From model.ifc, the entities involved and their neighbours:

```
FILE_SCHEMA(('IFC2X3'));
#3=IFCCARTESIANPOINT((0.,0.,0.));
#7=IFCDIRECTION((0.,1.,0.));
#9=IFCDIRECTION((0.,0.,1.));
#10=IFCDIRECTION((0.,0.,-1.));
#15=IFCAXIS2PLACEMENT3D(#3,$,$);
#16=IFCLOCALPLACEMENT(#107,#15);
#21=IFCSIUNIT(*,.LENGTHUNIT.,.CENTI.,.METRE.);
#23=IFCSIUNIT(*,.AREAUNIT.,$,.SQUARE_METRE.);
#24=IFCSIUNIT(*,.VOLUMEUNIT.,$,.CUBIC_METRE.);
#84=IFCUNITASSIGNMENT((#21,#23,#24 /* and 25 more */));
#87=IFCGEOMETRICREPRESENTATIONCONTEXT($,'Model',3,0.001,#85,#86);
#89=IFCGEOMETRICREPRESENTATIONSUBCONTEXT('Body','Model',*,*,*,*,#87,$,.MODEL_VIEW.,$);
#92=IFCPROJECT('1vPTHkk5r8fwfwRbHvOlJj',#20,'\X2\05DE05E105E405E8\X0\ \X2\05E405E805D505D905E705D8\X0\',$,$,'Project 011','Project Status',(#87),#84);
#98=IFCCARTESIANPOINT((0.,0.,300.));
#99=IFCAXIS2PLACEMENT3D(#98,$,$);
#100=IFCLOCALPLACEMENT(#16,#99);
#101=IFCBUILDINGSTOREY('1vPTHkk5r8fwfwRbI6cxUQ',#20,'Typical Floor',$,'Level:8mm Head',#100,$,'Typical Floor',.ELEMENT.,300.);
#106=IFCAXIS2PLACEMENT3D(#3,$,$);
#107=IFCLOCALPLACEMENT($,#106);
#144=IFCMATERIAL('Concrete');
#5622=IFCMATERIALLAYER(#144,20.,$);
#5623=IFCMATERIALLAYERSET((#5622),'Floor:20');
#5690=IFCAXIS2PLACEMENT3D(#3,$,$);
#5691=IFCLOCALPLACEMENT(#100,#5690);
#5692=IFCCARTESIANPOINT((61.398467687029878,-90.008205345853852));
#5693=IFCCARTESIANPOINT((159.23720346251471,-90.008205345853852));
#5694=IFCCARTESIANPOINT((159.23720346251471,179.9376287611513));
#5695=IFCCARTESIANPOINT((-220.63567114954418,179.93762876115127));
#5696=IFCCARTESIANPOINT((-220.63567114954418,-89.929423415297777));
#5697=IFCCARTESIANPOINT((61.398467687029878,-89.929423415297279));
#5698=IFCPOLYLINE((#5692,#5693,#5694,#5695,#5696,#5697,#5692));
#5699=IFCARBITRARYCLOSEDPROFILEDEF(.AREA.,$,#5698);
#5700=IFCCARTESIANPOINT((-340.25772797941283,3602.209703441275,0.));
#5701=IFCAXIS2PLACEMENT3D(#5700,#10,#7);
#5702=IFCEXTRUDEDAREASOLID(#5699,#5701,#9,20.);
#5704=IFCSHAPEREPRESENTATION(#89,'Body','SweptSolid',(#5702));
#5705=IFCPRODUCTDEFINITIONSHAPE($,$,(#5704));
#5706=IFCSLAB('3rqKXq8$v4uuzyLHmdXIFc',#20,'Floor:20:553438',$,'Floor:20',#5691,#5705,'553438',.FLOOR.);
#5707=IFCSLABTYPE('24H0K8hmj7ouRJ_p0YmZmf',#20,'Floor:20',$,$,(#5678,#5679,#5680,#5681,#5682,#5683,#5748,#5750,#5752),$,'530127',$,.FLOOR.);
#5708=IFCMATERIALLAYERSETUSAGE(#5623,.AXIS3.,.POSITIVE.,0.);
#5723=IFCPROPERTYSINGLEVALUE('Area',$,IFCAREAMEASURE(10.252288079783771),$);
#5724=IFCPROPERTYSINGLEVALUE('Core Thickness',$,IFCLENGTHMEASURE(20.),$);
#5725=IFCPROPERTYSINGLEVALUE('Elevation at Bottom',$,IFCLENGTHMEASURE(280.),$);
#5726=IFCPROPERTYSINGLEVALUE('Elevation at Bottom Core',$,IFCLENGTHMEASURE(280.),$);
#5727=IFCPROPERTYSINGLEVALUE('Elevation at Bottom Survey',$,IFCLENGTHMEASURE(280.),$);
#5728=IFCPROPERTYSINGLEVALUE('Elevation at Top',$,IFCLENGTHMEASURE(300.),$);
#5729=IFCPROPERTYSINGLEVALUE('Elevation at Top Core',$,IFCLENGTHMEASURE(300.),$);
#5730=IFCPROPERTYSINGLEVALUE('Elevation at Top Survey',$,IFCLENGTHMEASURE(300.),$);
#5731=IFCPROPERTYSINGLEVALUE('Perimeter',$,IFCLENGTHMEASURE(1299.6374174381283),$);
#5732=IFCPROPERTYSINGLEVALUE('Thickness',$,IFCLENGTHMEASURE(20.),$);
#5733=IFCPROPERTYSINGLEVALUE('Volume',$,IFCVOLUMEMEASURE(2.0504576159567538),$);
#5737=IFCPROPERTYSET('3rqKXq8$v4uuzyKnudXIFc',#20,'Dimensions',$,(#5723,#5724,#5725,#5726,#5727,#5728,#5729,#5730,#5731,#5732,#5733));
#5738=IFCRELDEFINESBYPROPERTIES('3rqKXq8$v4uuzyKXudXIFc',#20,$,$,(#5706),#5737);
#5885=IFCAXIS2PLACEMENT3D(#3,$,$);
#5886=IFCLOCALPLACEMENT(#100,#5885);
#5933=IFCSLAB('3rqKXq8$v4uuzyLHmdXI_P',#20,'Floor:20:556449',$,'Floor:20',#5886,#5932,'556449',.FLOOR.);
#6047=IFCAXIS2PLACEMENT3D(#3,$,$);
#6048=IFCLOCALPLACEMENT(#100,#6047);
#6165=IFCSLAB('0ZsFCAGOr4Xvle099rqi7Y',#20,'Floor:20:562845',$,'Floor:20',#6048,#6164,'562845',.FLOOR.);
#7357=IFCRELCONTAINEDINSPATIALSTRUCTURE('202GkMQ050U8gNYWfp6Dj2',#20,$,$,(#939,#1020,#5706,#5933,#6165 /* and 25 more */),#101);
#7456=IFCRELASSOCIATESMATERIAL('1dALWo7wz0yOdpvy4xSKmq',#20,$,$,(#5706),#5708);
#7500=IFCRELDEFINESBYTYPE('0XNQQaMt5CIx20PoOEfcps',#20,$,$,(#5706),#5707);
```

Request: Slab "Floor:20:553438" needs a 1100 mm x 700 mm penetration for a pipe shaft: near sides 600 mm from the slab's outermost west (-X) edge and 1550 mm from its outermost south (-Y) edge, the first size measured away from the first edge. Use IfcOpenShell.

```python
import numpy as np
import ifcopenshell
import ifcopenshell.api.feature
import ifcopenshell.api.geometry
import ifcopenshell.api.pset
import ifcopenshell.api.root
import ifcopenshell.geom
import ifcopenshell.util.element
import ifcopenshell.util.placement
import ifcopenshell.util.representation
import ifcopenshell.util.shape
import ifcopenshell.util.unit

model = ifcopenshell.open("model.ifc")
unit_scale = ifcopenshell.util.unit.calculate_unit_scale(model)
area_scale = ifcopenshell.util.unit.calculate_unit_scale(model, "AREAUNIT")
volume_scale = ifcopenshell.util.unit.calculate_unit_scale(model, "VOLUMEUNIT")
settings = ifcopenshell.geom.settings()


def volume(element):
    """Net volume in cubic metres, openings subtracted."""
    shape = ifcopenshell.geom.create_shape(settings, element)
    return ifcopenshell.util.shape.get_volume(shape.geometry)


slab = model.by_guid("3rqKXq8$v4uuzyLHmdXIFc")
before = volume(slab)

# Extent in the slab's own axes, in metres. The edges named are its -X and -Y sides.
slab_shape = ifcopenshell.geom.create_shape(settings, slab)
vertices = ifcopenshell.util.shape.get_vertices(slab_shape.geometry)
x_min, y_min, bottom = vertices.min(axis=0)
top = vertices[:, 2].max()

opening = ifcopenshell.api.root.create_entity(model, ifc_class="IfcOpeningElement", name="Pipe shaft opening")
context = ifcopenshell.util.representation.get_context(model, "Model", "Body", "MODEL_VIEW")
width, depth = 1.1, 0.7
outline = [(0.0, 0.0), (width, 0.0), (width, depth), (0.0, depth), (0.0, 0.0)]
# Overshoot both faces by 50 mm so the cut is clean.
shape = ifcopenshell.api.geometry.add_slab_representation(
    model, context=context, depth=top - bottom + 0.1, polyline=outline
)
ifcopenshell.api.geometry.assign_representation(model, product=opening, representation=shape)

matrix = ifcopenshell.util.placement.get_local_placement(slab.ObjectPlacement)
matrix[:, 3] = matrix @ np.append(np.array([x_min + 0.6, y_min + 1.55, bottom - 0.05]) / unit_scale, 1.0)
ifcopenshell.api.geometry.edit_object_placement(model, product=opening, matrix=matrix, is_si=False)
ifcopenshell.api.feature.add_feature(model, feature=opening, element=slab)

after = volume(slab)

# Update the slab's stored quantities.
pset = model.by_id(ifcopenshell.util.element.get_pset(slab, "Dimensions", should_inherit=False)["id"])
ifcopenshell.api.pset.edit_pset(model, pset=pset, properties={
    "Area": model.create_entity("IfcAreaMeasure", after / (top - bottom) / area_scale),
    "Volume": model.create_entity("IfcVolumeMeasure", after / volume_scale),
})

print(f"slab volume {before:.3f} -> {after:.3f} m3")

model.write("model_updated.ifc")
```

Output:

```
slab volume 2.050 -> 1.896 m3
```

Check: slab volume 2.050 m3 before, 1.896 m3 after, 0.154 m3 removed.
